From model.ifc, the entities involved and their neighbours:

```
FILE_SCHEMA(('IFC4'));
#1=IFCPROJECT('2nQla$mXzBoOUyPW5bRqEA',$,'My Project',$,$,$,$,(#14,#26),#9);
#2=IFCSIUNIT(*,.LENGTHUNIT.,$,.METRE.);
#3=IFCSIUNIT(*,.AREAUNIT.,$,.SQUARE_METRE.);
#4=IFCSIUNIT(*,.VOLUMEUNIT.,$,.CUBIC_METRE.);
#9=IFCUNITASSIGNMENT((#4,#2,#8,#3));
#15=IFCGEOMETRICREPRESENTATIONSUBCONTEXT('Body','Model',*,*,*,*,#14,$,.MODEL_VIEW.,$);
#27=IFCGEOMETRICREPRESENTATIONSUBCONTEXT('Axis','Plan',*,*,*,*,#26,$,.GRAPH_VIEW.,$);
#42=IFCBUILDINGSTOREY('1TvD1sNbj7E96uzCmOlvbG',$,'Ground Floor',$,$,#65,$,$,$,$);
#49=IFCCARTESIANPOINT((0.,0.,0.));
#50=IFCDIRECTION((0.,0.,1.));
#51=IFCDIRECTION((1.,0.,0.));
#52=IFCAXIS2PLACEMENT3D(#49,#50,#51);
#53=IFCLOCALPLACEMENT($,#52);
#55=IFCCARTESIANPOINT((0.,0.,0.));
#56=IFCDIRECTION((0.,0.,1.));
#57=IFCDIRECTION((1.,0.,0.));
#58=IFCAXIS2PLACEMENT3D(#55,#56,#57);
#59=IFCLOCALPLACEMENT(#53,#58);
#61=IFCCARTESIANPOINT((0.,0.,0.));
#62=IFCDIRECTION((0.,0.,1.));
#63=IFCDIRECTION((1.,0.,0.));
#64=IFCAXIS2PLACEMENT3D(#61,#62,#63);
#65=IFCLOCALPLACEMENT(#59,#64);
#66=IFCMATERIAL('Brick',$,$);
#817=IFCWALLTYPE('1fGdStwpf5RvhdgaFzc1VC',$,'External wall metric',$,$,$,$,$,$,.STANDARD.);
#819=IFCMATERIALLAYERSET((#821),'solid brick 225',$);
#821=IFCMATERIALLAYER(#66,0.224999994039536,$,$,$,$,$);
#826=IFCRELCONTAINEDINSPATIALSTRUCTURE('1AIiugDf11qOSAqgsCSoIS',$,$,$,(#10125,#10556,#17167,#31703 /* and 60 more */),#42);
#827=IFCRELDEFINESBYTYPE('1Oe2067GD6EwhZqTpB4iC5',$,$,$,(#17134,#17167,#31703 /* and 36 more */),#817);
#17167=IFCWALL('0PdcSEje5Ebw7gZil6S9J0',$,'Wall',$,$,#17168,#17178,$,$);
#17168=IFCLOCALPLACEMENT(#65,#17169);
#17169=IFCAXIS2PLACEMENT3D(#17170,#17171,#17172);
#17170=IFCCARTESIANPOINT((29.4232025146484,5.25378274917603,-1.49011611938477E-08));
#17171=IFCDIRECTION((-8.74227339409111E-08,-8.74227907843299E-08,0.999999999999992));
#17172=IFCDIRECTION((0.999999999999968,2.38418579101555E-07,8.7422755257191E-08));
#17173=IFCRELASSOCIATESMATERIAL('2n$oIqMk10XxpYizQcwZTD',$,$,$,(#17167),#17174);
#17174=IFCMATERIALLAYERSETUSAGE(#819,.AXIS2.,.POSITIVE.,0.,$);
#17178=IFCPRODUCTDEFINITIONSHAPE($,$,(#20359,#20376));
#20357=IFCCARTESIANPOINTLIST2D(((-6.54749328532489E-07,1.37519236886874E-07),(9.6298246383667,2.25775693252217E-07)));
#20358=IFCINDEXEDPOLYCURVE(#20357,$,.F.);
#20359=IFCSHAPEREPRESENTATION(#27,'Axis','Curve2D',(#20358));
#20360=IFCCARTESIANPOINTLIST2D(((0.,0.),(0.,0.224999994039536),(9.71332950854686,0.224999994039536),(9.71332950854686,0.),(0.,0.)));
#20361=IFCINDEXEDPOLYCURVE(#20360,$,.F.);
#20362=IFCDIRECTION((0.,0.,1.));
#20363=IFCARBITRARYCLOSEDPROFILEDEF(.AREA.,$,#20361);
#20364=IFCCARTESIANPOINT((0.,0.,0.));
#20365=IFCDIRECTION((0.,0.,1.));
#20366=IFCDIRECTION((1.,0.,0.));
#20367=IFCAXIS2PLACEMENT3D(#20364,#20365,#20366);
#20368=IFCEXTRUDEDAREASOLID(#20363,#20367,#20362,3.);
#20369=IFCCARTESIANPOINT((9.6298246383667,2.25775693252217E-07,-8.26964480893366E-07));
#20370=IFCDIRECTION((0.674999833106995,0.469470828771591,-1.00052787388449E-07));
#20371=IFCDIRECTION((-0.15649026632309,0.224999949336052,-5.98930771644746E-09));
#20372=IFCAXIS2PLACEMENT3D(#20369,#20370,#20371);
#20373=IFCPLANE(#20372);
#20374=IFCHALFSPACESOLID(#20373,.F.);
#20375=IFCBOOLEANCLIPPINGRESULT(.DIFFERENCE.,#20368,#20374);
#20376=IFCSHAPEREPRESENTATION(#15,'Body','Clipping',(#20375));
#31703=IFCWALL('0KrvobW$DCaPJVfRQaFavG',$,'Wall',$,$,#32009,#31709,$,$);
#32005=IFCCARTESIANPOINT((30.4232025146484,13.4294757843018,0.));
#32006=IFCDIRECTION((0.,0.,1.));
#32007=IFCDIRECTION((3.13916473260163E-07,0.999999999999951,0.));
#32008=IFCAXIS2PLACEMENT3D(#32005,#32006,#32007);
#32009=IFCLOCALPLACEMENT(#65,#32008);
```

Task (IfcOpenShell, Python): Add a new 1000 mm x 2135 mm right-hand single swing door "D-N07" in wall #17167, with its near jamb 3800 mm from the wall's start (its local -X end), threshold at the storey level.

```python
import numpy as np
import ifcopenshell
import ifcopenshell.api.feature
import ifcopenshell.api.geometry
import ifcopenshell.api.root
import ifcopenshell.api.spatial
import ifcopenshell.geom
import ifcopenshell.util.element
import ifcopenshell.util.placement
import ifcopenshell.util.representation
import ifcopenshell.util.shape
import ifcopenshell.util.unit

model = ifcopenshell.open("model.ifc")
unit_scale = ifcopenshell.util.unit.calculate_unit_scale(model)
settings = ifcopenshell.geom.settings()


def volume(element):
    """Net volume in cubic metres, openings subtracted."""
    shape = ifcopenshell.geom.create_shape(settings, element)
    return ifcopenshell.util.shape.get_volume(shape.geometry)


wall = model.by_id(17167)
storey = ifcopenshell.util.element.get_container(wall, ifc_class="IfcBuildingStorey")
context = ifcopenshell.util.representation.get_context(model, "Model", "Body", "MODEL_VIEW")
before = volume(wall)

width, height, from_end, sill = 1, 2.135, 3.8, 0.0  # metres

# The wall runs along its own X axis, and the end named is its -X end.
wall_shape = ifcopenshell.geom.create_shape(settings, wall)
x, y, z = ifcopenshell.util.shape.get_vertices(wall_shape.geometry).T
start = x.min() + from_end
face, thickness = float(y.min()), float(y.max() - y.min())
wall_matrix = ifcopenshell.util.placement.get_local_placement(wall.ObjectPlacement)
level = ifcopenshell.util.placement.get_local_placement(storey.ObjectPlacement)[2, 3]


def in_wall(x, y):
    """Placement at x, y metres in the wall's axes, at sill height."""
    matrix = wall_matrix.copy()
    matrix[:, 3] = wall_matrix @ np.array([x / unit_scale, y / unit_scale, 0.0, 1.0])
    matrix[2, 3] = level + sill / unit_scale
    return matrix


# Opening: a box that overshoots both wall faces by 50 mm.
opening = ifcopenshell.api.root.create_entity(model, ifc_class="IfcOpeningElement", predefined_type="OPENING")
box = ifcopenshell.api.geometry.add_wall_representation(
    model, context=context, length=width, height=height, thickness=thickness + 0.1
)
ifcopenshell.api.geometry.assign_representation(model, product=opening, representation=box)
ifcopenshell.api.geometry.edit_object_placement(model, product=opening, matrix=in_wall(start, face - 0.05), is_si=False)
ifcopenshell.api.feature.add_feature(model, feature=opening, element=wall)

door = ifcopenshell.api.root.create_entity(model, ifc_class="IfcDoor", name="D-N07", predefined_type="DOOR")
door.OverallWidth, door.OverallHeight = width / unit_scale, height / unit_scale
door.OperationType = "SINGLE_SWING_RIGHT"
body = ifcopenshell.api.geometry.add_door_representation(
    model,
    context=context,
    overall_width=door.OverallWidth,
    overall_height=door.OverallHeight,
    operation_type="SINGLE_SWING_RIGHT",
    lining_properties={"LiningDepth": thickness / unit_scale, "ThresholdDepth": thickness / unit_scale},
)
ifcopenshell.api.geometry.assign_representation(model, product=door, representation=body)
ifcopenshell.api.spatial.assign_container(model, products=[door], relating_structure=storey)
ifcopenshell.api.feature.add_filling(model, opening=opening, element=door)

# The lining spans the wall, so the door starts at the wall face.
ifcopenshell.api.geometry.edit_object_placement(model, product=door, matrix=in_wall(start, face), is_si=False)

after = volume(wall)

print(f"wall volume {before:.3f} -> {after:.3f} m3")

model.write("model_edited.ifc")
```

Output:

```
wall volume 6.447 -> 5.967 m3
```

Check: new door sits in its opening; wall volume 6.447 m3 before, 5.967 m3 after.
